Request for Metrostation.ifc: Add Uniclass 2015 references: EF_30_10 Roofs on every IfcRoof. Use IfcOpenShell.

First a look at what the model holds.

```python
import ifcopenshell

model = ifcopenshell.open("Metrostation.ifc")
print(model.schema)
print("classifications:", [c.Name for c in model.by_type("IfcClassification")])
for ifc_class in ("IfcDoor", "IfcRoof", "IfcStair", "IfcWall", "IfcWindow"):
    print(ifc_class, len(model.by_type(ifc_class)))
```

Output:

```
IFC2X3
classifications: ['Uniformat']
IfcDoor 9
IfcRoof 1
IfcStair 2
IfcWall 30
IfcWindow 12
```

```python
import ifcopenshell
import ifcopenshell.api.classification

model = ifcopenshell.open("Metrostation.ifc")

# IFC2X3 requires Source and Edition and has no link from the project to the system.
system = model.create_entity("IfcClassification", Source="NBS", Edition="2015", Name="Uniclass 2015")

codes = {
    "IfcRoof": ("EF_30_10", "Roofs"),
}
for ifc_class, (code, name) in codes.items():
    products = model.by_type(ifc_class)
    ifcopenshell.api.classification.add_reference(
        model, products=products, classification=system, identification=code, name=name
    )
    print(code, len(products))

model.write("Metrostation_edited.ifc")
```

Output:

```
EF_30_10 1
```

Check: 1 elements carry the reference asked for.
